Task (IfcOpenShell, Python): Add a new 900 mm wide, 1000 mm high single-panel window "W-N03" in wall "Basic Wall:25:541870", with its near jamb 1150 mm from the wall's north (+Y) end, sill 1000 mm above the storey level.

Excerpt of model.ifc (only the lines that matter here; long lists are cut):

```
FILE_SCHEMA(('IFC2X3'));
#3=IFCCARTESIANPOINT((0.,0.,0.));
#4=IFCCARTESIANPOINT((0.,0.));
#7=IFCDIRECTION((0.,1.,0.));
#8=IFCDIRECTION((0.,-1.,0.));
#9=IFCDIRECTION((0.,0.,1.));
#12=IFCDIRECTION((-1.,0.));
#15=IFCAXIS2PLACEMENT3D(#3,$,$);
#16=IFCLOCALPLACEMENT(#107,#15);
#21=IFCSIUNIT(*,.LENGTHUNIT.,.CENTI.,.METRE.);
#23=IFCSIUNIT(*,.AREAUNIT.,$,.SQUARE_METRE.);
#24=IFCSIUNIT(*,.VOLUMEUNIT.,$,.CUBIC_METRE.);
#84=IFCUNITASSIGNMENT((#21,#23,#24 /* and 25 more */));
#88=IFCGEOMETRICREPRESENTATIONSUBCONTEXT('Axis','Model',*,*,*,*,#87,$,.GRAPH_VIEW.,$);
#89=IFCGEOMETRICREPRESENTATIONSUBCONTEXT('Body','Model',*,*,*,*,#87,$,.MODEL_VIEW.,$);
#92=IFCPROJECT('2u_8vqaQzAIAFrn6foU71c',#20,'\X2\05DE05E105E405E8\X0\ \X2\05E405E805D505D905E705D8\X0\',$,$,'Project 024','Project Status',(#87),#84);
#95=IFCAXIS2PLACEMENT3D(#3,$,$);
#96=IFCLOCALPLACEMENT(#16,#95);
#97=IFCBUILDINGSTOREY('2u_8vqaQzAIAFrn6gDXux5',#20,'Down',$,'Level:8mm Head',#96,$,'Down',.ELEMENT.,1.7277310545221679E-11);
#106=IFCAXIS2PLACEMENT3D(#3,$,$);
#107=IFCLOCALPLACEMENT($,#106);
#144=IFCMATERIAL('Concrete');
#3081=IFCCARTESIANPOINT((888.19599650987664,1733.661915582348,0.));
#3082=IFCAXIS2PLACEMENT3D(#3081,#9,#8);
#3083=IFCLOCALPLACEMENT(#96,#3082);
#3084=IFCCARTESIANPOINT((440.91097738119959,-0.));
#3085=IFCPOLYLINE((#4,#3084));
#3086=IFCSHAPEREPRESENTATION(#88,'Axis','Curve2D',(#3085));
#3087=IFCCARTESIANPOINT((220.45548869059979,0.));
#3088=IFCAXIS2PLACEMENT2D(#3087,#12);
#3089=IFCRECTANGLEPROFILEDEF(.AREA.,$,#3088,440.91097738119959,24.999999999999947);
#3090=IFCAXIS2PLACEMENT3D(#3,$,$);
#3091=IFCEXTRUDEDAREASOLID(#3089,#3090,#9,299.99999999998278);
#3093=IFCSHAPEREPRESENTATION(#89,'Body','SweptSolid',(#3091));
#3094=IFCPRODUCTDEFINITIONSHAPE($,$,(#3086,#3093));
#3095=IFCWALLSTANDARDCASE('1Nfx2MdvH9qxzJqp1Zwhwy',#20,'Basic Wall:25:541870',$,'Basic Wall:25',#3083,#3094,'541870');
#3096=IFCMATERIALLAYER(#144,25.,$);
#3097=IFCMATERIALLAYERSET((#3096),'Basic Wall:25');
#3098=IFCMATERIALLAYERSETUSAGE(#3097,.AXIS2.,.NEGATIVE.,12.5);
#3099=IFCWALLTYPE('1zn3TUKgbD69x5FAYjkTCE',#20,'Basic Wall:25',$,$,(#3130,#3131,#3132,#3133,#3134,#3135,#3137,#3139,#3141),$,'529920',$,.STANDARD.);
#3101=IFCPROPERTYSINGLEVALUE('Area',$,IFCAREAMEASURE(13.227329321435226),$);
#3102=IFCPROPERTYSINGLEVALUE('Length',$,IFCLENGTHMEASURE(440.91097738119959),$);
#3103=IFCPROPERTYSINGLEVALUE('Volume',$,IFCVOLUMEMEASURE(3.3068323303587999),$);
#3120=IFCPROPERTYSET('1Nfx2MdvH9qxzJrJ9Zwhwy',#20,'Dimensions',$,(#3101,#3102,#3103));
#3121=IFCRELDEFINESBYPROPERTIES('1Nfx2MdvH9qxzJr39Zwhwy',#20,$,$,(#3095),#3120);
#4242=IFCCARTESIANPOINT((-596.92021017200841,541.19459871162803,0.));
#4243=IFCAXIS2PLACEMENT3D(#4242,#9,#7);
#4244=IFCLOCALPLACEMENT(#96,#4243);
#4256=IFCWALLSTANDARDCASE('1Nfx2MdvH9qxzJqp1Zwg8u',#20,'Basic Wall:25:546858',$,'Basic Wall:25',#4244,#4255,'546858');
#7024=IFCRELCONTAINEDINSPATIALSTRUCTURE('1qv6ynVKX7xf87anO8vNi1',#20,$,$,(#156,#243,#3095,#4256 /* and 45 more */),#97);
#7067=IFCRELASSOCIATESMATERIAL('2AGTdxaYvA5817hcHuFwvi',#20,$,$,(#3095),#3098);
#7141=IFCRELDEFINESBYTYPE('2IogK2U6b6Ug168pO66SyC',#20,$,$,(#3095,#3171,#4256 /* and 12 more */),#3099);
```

```python
import numpy as np
import ifcopenshell
import ifcopenshell.api.feature
import ifcopenshell.api.geometry
import ifcopenshell.api.pset
import ifcopenshell.api.root
import ifcopenshell.api.spatial
import ifcopenshell.api.type
import ifcopenshell.geom
import ifcopenshell.util.element
import ifcopenshell.util.placement
import ifcopenshell.util.representation
import ifcopenshell.util.shape
import ifcopenshell.util.unit

model = ifcopenshell.open("model.ifc")
unit_scale = ifcopenshell.util.unit.calculate_unit_scale(model)
area_scale = ifcopenshell.util.unit.calculate_unit_scale(model, "AREAUNIT")
volume_scale = ifcopenshell.util.unit.calculate_unit_scale(model, "VOLUMEUNIT")
settings = ifcopenshell.geom.settings()


def volume(element):
    """Net volume in cubic metres, openings subtracted."""
    shape = ifcopenshell.geom.create_shape(settings, element)
    return ifcopenshell.util.shape.get_volume(shape.geometry)


wall = model.by_id(3095)
storey = ifcopenshell.util.element.get_container(wall, ifc_class="IfcBuildingStorey")
context = ifcopenshell.util.representation.get_context(model, "Model", "Body", "MODEL_VIEW")
before = volume(wall)

width, height, from_end, sill = 0.9, 1, 1.15, 1  # metres

# The wall runs along its own X axis, and the end named is its -X end.
wall_shape = ifcopenshell.geom.create_shape(settings, wall)
x, y, z = ifcopenshell.util.shape.get_vertices(wall_shape.geometry).T
start = x.min() + from_end
face, thickness = float(y.min()), float(y.max() - y.min())
wall_matrix = ifcopenshell.util.placement.get_local_placement(wall.ObjectPlacement)
level = ifcopenshell.util.placement.get_local_placement(storey.ObjectPlacement)[2, 3]


def in_wall(x, y):
    """Placement at x, y metres in the wall's axes, at sill height."""
    matrix = wall_matrix.copy()
    matrix[:, 3] = wall_matrix @ np.array([x / unit_scale, y / unit_scale, 0.0, 1.0])
    matrix[2, 3] = level + sill / unit_scale
    return matrix


# Opening: a box that overshoots both wall faces by 50 mm.
opening = ifcopenshell.api.root.create_entity(model, ifc_class="IfcOpeningElement")
box = ifcopenshell.api.geometry.add_wall_representation(
    model, context=context, length=width, height=height, thickness=thickness + 0.1
)
ifcopenshell.api.geometry.assign_representation(model, product=opening, representation=box)
ifcopenshell.api.geometry.edit_object_placement(model, product=opening, matrix=in_wall(start, face - 0.05), is_si=False)
ifcopenshell.api.feature.add_feature(model, feature=opening, element=wall)

window = ifcopenshell.api.root.create_entity(model, ifc_class="IfcWindow", name="W-N03")
window.OverallWidth, window.OverallHeight = width / unit_scale, height / unit_scale
body = ifcopenshell.api.geometry.add_window_representation(
    model,
    context=context,
    overall_width=window.OverallWidth,
    overall_height=window.OverallHeight,
    partition_type="SINGLE_PANEL",
)
ifcopenshell.api.geometry.assign_representation(model, product=window, representation=body)
ifcopenshell.api.spatial.assign_container(model, products=[window], relating_structure=storey)
fills = ifcopenshell.api.feature.add_filling(model, opening=opening, element=window)
fills.OwnerHistory = window.OwnerHistory  # required in IFC2X3

# IFC2X3 keeps the operation on the window style.
style = ifcopenshell.api.root.create_entity(model, ifc_class="IfcWindowStyle", name="W-N03")
style.OperationType, style.ConstructionType = "SINGLE_PANEL", "NOTDEFINED"
style.ParameterTakesPrecedence = style.Sizeable = False
ifcopenshell.api.type.assign_type(model, related_objects=[window], relating_type=style)

# Centre the window in the wall's thickness.
ifcopenshell.api.geometry.edit_object_placement(model, product=window, matrix=in_wall(start, face), is_si=False)
window_shape = ifcopenshell.geom.create_shape(settings, window)
depth = ifcopenshell.util.shape.get_vertices(window_shape.geometry)[:, 1]
offset = face + thickness / 2 - (depth.min() + depth.max()) / 2
ifcopenshell.api.geometry.edit_object_placement(model, product=window, matrix=in_wall(start, offset), is_si=False)

after = volume(wall)

# Update the wall's stored quantities.
pset = model.by_id(ifcopenshell.util.element.get_pset(wall, "Dimensions", should_inherit=False)["id"])
ifcopenshell.api.pset.edit_pset(model, pset=pset, properties={
    "Area": model.create_entity("IfcAreaMeasure", after / thickness / area_scale),
    "Volume": model.create_entity("IfcVolumeMeasure", after / volume_scale),
})

print(f"wall volume {before:.3f} -> {after:.3f} m3")

model.write("model_rev.ifc")
```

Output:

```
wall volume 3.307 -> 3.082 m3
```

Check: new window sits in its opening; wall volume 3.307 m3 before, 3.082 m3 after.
